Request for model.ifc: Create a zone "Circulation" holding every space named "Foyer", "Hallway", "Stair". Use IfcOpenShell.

First a look at what the model holds.

```python
import ifcopenshell

model = ifcopenshell.open("model.ifc")
print(model.schema)
seen = {}
for space in model.by_type("IfcSpace"):
    seen[space.LongName] = seen.get(space.LongName, 0) + 1
for name, count in sorted(seen.items(), key=str):
    print(count, "x", name)
print("zones:", [z.Name for z in model.by_type("IfcZone")][:20])
```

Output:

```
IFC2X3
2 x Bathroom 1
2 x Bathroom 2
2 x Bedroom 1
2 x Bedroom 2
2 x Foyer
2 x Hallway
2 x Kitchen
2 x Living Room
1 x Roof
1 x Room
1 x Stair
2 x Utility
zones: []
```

```python
import ifcopenshell
import ifcopenshell.api.group
import ifcopenshell.api.root

model = ifcopenshell.open("model.ifc")

names = {"Foyer", "Hallway", "Stair"}
spaces = [s for s in model.by_type("IfcSpace") if s.LongName in names]

zone = ifcopenshell.api.root.create_entity(model, ifc_class="IfcZone", name="Circulation")
ifcopenshell.api.group.assign_group(model, products=spaces, group=zone)
print(len(spaces), "spaces in", zone.Name)

model.write("model_edited.ifc")
```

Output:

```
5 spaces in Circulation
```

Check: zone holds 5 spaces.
